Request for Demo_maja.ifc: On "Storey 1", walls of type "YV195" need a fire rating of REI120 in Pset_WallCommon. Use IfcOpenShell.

First a look at what the model holds.

```python
import ifcopenshell
import ifcopenshell.util.element

model = ifcopenshell.open("Demo_maja.ifc")
print(model.schema)
storey = next(s for s in model.by_type("IfcBuildingStorey") if s.Name == "Storey 1")
walls = [e for e in ifcopenshell.util.element.get_decomposition(storey) if e.is_a("IfcWall")]
seen = {}
for e in walls:
    element_type = ifcopenshell.util.element.get_type(e)
    key = (element_type.Name if element_type != e and element_type else None, ifcopenshell.util.element.get_pset(e, "Pset_WallCommon", "FireRating"))
    seen[key] = seen.get(key, 0) + 1
for (name, value), count in sorted(seen.items(), key=str):
    print(count, "x", name, "|", value)
```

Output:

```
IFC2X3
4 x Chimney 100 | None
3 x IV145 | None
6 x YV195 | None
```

```python
import ifcopenshell
import ifcopenshell.api.pset
import ifcopenshell.util.element

model = ifcopenshell.open("Demo_maja.ifc")

storey = next(s for s in model.by_type("IfcBuildingStorey") if s.Name == "Storey 1")
walls = [e for e in ifcopenshell.util.element.get_decomposition(storey) if e.is_a("IfcWall")]

count = 0
for e in walls:
    element_type = ifcopenshell.util.element.get_type(e)
    if element_type in (None, e) or element_type.Name != "YV195":
        continue
    # add_pset returns the element's existing set when there is one.
    pset = ifcopenshell.api.pset.add_pset(model, product=e, name="Pset_WallCommon")
    ifcopenshell.api.pset.edit_pset(model, pset=pset, properties={"FireRating": "REI120"})
    count += 1

print(count, "walls updated")

model.write("Demo_maja-out.ifc")
```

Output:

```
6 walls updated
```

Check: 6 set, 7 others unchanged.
